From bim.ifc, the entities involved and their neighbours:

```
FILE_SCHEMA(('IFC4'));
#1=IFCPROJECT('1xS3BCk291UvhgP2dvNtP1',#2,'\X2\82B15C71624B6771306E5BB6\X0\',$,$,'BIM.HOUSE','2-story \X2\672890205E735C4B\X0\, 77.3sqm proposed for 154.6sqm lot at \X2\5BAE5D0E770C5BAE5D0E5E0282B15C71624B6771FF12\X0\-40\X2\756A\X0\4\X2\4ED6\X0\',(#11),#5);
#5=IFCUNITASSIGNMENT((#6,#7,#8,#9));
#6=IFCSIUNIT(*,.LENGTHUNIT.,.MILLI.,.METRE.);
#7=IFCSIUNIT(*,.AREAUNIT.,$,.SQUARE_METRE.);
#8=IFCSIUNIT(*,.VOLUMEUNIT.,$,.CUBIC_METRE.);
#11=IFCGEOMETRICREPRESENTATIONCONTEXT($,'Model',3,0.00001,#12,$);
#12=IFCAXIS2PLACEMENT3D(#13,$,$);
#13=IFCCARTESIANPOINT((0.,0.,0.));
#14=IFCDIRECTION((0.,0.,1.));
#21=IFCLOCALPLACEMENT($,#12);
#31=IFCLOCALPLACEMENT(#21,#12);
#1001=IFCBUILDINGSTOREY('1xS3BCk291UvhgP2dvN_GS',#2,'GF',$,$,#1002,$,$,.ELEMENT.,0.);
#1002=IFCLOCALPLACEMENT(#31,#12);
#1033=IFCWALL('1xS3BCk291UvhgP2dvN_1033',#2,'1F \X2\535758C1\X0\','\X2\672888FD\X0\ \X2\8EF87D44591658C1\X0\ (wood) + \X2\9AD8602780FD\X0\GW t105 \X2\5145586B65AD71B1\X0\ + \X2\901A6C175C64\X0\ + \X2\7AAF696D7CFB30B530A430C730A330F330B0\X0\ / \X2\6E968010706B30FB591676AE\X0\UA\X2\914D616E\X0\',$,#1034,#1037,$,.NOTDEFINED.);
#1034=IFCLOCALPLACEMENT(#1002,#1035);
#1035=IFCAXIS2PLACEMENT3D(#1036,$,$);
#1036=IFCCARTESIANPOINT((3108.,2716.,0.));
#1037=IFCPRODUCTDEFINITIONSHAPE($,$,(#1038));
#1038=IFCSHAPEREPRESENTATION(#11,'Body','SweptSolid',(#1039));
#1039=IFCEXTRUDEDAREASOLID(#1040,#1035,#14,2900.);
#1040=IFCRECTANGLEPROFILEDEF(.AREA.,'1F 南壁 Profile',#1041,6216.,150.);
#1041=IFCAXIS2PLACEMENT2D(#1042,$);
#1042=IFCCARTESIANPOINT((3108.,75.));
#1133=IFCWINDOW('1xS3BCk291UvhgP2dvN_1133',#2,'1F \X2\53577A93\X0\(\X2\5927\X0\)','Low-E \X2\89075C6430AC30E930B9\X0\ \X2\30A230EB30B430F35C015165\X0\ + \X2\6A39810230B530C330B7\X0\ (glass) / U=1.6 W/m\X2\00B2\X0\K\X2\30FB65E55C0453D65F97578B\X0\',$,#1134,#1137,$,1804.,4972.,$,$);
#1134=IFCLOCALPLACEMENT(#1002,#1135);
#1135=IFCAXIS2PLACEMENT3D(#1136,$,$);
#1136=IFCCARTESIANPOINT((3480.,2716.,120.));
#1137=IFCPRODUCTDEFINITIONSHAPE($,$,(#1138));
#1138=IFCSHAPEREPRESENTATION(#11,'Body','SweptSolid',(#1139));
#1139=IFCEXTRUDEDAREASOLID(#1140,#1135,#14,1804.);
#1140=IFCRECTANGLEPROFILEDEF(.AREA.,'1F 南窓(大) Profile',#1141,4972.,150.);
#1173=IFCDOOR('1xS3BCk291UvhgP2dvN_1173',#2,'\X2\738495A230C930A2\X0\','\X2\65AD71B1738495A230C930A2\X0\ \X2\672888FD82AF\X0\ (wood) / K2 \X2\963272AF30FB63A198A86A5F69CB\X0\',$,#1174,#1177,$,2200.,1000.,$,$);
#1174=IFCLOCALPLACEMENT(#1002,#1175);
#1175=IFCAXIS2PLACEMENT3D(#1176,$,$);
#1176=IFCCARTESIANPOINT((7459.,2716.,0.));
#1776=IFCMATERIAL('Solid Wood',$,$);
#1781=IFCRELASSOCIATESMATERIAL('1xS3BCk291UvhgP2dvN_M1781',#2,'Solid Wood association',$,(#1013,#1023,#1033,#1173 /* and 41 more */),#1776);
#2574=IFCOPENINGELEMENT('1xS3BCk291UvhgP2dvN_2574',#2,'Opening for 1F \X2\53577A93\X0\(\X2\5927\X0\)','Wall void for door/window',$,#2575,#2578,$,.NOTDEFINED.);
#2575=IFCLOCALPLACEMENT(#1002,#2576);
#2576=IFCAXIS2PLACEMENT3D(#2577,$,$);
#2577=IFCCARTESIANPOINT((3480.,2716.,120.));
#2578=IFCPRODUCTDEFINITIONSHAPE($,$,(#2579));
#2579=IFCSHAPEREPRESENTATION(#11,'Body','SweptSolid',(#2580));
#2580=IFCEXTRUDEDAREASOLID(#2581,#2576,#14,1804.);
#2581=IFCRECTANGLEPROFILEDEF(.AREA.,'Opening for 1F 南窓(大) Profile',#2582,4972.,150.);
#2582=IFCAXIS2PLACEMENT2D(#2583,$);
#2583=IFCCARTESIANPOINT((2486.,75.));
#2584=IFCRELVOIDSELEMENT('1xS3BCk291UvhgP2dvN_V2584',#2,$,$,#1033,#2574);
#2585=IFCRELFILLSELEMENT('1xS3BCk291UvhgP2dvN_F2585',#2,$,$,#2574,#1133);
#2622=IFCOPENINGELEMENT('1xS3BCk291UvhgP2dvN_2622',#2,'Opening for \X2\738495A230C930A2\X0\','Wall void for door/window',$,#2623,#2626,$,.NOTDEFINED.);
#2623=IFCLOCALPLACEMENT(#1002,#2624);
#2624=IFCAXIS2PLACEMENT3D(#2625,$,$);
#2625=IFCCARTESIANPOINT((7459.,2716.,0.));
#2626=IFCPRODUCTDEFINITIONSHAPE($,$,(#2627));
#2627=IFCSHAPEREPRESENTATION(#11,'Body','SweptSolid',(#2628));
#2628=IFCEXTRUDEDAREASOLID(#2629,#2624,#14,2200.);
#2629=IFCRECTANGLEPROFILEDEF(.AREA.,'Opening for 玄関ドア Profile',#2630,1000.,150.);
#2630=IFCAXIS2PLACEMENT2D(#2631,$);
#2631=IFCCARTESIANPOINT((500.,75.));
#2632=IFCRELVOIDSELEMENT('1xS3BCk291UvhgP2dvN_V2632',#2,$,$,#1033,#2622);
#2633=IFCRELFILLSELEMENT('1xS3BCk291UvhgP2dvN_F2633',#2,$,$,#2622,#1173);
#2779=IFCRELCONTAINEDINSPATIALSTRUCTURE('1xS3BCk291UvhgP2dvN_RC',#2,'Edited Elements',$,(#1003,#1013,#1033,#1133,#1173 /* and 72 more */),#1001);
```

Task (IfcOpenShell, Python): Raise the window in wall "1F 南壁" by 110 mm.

```python
import numpy as np
import ifcopenshell
import ifcopenshell.api.geometry
import ifcopenshell.util.placement
import ifcopenshell.util.unit

model = ifcopenshell.open("bim.ifc")
unit_scale = ifcopenshell.util.unit.calculate_unit_scale(model)

window = model.by_guid("1xS3BCk291UvhgP2dvN_1133")
opening = window.FillsVoids[0].RelatingOpeningElement
dz = 0.11 / unit_scale

shift = np.array([0.0, 0.0, dz])
# The window is not placed relative to its opening, so move both.
for product in (opening, window):
    matrix = ifcopenshell.util.placement.get_local_placement(product.ObjectPlacement)
    matrix[:3, 3] += shift
    ifcopenshell.api.geometry.edit_object_placement(model, product=product, matrix=matrix, is_si=False)

print(f"moved by {dz * unit_scale:+.3f} m")

model.write("bim_v2.ifc")
```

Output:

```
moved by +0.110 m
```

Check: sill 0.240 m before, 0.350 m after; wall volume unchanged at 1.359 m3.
